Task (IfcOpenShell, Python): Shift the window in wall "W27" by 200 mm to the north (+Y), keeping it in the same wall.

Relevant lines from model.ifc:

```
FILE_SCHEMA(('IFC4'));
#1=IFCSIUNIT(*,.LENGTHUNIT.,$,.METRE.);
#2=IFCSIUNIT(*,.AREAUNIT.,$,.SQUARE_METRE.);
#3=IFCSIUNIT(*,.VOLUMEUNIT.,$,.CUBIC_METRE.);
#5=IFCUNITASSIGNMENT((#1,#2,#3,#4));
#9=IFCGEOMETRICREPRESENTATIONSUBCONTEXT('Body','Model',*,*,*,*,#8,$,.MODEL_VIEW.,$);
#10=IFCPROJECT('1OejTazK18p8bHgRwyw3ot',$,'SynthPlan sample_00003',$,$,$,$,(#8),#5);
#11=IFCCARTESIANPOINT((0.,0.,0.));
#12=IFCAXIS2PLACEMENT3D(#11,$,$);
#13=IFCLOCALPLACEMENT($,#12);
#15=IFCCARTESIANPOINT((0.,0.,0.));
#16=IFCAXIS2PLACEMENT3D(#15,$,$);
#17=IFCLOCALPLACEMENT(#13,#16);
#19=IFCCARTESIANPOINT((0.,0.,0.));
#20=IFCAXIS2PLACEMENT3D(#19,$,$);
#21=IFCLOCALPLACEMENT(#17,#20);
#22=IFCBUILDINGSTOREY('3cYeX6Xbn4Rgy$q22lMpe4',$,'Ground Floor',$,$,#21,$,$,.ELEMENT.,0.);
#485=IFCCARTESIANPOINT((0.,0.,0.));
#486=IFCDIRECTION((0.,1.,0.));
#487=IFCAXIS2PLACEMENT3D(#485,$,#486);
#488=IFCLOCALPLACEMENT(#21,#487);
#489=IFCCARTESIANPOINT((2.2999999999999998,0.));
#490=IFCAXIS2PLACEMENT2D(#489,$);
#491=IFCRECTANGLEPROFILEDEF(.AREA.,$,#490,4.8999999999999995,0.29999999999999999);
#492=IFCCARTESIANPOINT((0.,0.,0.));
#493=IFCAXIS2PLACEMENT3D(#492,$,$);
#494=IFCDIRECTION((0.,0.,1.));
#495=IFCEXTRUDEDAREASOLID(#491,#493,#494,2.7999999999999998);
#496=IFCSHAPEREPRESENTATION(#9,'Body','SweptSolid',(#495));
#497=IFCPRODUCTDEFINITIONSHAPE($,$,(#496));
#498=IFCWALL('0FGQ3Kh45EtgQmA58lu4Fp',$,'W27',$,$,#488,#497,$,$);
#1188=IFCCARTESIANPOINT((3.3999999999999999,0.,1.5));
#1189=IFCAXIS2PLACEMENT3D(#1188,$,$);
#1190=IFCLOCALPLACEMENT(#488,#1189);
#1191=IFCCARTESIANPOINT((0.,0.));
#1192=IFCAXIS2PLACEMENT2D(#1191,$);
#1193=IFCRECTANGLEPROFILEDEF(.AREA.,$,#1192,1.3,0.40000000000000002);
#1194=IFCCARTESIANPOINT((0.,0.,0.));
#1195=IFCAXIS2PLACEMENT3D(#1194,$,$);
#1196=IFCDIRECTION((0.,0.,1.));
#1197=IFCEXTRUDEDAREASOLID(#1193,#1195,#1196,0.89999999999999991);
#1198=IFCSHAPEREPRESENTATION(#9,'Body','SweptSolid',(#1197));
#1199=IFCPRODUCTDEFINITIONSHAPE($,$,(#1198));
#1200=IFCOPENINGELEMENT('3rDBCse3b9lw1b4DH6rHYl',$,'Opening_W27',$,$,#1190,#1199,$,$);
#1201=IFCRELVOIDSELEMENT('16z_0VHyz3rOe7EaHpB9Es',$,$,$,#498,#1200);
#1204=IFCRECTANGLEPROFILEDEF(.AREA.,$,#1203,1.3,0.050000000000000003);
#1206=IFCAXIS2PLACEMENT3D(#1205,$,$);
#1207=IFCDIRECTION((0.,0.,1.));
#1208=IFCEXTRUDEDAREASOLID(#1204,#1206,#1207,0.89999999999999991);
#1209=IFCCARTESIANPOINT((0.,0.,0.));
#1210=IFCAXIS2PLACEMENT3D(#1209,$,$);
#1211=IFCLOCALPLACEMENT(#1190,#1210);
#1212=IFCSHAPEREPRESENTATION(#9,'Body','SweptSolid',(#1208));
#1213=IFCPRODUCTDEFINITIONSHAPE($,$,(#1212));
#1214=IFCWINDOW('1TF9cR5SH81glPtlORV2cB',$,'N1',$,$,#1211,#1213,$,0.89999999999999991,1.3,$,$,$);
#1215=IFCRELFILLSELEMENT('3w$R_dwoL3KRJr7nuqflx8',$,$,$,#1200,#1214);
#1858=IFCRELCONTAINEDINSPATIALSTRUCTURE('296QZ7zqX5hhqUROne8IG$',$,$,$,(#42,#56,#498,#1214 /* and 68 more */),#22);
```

```python
import ifcopenshell
import ifcopenshell.api.geometry
import ifcopenshell.util.placement
import ifcopenshell.util.unit

model = ifcopenshell.open("model.ifc")
unit_scale = ifcopenshell.util.unit.calculate_unit_scale(model)

window = model.by_guid("1TF9cR5SH81glPtlORV2cB")
opening = window.FillsVoids[0].RelatingOpeningElement
wall = opening.VoidsElements[0].RelatingBuildingElement

wall_matrix = ifcopenshell.util.placement.get_local_placement(wall.ObjectPlacement)
shift = wall_matrix[:3, 0] * 0.2 / unit_scale
before = ifcopenshell.util.placement.get_local_placement(window.ObjectPlacement)[:3, 3].copy()

# The window is placed relative to its opening, so it follows when the opening moves.
matrix = ifcopenshell.util.placement.get_local_placement(opening.ObjectPlacement)
matrix[:3, 3] += shift
ifcopenshell.api.geometry.edit_object_placement(
    model, product=opening, matrix=matrix, is_si=False, should_transform_children=True
)

after = ifcopenshell.util.placement.get_local_placement(window.ObjectPlacement)[:3, 3]
print("window moved by", (after - before).round(3) + 0.0)

model.write("model_edited.ifc")
```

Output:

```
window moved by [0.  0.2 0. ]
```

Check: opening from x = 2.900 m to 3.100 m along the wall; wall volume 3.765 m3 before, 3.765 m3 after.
